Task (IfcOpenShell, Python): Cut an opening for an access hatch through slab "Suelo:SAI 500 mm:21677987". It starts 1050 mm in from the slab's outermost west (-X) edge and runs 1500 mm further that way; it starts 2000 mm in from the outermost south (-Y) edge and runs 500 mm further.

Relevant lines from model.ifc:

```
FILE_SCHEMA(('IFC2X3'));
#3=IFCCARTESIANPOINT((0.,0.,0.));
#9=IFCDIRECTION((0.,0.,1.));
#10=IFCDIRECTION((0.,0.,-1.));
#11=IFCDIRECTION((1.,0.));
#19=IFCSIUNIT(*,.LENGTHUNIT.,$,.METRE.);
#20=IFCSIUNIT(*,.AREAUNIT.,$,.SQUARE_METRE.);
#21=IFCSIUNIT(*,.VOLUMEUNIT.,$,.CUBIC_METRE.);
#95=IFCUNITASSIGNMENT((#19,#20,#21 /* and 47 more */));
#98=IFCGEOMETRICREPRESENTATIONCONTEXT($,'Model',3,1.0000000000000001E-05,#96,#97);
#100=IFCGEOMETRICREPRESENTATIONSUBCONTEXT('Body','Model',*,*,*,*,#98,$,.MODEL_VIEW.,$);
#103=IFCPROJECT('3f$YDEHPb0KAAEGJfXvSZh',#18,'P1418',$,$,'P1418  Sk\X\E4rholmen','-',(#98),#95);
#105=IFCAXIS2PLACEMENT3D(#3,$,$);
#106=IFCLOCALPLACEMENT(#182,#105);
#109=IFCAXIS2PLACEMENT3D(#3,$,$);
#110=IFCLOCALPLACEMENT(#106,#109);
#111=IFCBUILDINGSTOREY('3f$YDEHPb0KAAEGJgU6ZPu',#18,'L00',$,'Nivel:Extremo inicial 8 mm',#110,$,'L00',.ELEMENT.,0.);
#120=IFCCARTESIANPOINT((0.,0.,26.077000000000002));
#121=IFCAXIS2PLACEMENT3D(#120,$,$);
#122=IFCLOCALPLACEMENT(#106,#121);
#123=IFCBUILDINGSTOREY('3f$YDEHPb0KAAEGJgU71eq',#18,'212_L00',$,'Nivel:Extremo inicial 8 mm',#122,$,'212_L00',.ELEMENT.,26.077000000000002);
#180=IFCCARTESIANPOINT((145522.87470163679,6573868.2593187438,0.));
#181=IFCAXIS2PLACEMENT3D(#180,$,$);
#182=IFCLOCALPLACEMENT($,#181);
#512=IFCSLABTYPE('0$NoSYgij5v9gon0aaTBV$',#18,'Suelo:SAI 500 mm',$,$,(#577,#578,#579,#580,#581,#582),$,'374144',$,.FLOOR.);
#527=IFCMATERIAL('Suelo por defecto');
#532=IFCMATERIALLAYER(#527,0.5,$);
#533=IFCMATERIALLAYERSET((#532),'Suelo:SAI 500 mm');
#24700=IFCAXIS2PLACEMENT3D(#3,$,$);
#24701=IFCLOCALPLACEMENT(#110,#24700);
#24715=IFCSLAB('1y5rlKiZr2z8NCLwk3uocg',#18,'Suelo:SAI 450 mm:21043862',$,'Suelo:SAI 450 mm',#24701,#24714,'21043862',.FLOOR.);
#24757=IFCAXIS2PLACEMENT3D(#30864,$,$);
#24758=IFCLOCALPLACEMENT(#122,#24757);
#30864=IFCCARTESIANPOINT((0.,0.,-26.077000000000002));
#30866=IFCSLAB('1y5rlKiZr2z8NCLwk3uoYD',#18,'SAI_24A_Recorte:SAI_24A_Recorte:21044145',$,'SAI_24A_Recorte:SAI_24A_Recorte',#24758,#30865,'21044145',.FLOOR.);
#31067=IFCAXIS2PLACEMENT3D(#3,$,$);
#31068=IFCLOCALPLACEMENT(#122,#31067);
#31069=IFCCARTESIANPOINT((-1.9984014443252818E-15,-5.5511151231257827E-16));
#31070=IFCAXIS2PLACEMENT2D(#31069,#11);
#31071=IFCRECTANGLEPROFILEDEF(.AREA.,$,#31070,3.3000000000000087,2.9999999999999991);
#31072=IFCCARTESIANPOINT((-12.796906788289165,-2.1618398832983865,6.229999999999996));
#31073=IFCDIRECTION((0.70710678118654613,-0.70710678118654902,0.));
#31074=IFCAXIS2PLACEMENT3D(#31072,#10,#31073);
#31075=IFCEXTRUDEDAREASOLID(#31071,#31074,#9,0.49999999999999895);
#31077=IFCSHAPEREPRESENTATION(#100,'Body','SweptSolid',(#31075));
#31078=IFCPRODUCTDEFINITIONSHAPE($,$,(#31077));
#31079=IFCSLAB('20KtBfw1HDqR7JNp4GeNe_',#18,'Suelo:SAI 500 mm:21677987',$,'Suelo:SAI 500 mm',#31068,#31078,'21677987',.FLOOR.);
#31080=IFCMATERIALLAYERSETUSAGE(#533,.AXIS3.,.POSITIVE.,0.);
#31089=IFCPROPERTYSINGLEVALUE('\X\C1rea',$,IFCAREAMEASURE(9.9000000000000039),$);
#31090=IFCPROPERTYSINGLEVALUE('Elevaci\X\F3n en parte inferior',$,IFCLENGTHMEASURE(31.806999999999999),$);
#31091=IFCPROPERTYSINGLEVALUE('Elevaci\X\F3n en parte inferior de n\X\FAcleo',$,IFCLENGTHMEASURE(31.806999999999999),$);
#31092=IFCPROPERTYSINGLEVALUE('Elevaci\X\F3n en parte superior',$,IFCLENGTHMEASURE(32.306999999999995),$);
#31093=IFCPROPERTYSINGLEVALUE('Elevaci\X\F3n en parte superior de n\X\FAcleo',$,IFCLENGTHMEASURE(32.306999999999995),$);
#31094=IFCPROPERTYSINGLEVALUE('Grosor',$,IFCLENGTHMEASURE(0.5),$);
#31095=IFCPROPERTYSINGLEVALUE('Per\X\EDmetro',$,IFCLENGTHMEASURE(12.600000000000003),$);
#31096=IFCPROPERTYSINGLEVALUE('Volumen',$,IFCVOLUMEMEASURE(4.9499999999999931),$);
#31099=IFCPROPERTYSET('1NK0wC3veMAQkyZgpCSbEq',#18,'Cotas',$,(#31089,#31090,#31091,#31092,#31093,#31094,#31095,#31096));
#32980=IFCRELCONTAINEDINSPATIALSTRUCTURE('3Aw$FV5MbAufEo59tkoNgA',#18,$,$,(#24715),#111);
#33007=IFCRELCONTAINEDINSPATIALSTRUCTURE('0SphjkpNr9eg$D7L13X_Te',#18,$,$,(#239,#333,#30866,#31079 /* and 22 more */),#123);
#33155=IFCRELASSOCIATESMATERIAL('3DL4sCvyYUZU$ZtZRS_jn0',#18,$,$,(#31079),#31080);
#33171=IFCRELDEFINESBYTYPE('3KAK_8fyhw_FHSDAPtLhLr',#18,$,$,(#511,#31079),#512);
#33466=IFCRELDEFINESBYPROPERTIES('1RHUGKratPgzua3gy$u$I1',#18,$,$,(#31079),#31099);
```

```python
import numpy as np
import ifcopenshell
import ifcopenshell.api.feature
import ifcopenshell.api.geometry
import ifcopenshell.api.pset
import ifcopenshell.api.root
import ifcopenshell.geom
import ifcopenshell.util.element
import ifcopenshell.util.placement
import ifcopenshell.util.representation
import ifcopenshell.util.shape
import ifcopenshell.util.unit

model = ifcopenshell.open("model.ifc")
unit_scale = ifcopenshell.util.unit.calculate_unit_scale(model)
area_scale = ifcopenshell.util.unit.calculate_unit_scale(model, "AREAUNIT")
volume_scale = ifcopenshell.util.unit.calculate_unit_scale(model, "VOLUMEUNIT")
settings = ifcopenshell.geom.settings()


def volume(element):
    """Net volume in cubic metres, openings subtracted."""
    shape = ifcopenshell.geom.create_shape(settings, element)
    return ifcopenshell.util.shape.get_volume(shape.geometry)


slab = model.by_guid("20KtBfw1HDqR7JNp4GeNe_")
before = volume(slab)

# Extent in the slab's own axes, in metres. The edges named are its -X and -Y sides.
slab_shape = ifcopenshell.geom.create_shape(settings, slab)
vertices = ifcopenshell.util.shape.get_vertices(slab_shape.geometry)
x_min, y_min, bottom = vertices.min(axis=0)
top = vertices[:, 2].max()

opening = ifcopenshell.api.root.create_entity(model, ifc_class="IfcOpeningElement", name="Access hatch opening")
context = ifcopenshell.util.representation.get_context(model, "Model", "Body", "MODEL_VIEW")
width, depth = 1.5, 0.5
outline = [(0.0, 0.0), (width, 0.0), (width, depth), (0.0, depth), (0.0, 0.0)]
# Overshoot both faces by 50 mm so the cut is clean.
shape = ifcopenshell.api.geometry.add_slab_representation(
    model, context=context, depth=top - bottom + 0.1, polyline=outline
)
ifcopenshell.api.geometry.assign_representation(model, product=opening, representation=shape)

matrix = ifcopenshell.util.placement.get_local_placement(slab.ObjectPlacement)
matrix[:, 3] = matrix @ np.append(np.array([x_min + 1.05, y_min + 2, bottom - 0.05]) / unit_scale, 1.0)
ifcopenshell.api.geometry.edit_object_placement(model, product=opening, matrix=matrix, is_si=False)
ifcopenshell.api.feature.add_feature(model, feature=opening, element=slab)

after = volume(slab)

# Update the slab's stored quantities.
pset = model.by_id(ifcopenshell.util.element.get_pset(slab, "Cotas", should_inherit=False)["id"])
ifcopenshell.api.pset.edit_pset(model, pset=pset, properties={
    "Área": model.create_entity("IfcAreaMeasure", after / (top - bottom) / area_scale),
    "Volumen": model.create_entity("IfcVolumeMeasure", after / volume_scale),
})

print(f"slab volume {before:.3f} -> {after:.3f} m3")

model.write("model_rev.ifc")
```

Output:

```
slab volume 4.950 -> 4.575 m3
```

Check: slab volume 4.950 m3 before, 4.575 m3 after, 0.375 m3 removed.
